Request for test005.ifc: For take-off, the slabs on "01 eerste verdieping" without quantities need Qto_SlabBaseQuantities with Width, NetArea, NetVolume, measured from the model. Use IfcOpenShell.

First a look at what the model holds.

```python
import ifcopenshell
import ifcopenshell.util.element
import ifcopenshell.util.unit

model = ifcopenshell.open("test005.ifc")
print(model.schema)
for unit_type in ("LENGTHUNIT", "AREAUNIT", "VOLUMEUNIT"):
    print(unit_type, ifcopenshell.util.unit.calculate_unit_scale(model, unit_type))
storey = next(s for s in model.by_type("IfcBuildingStorey") if s.Name == "01 eerste verdieping")
slabs = [e for e in ifcopenshell.util.element.get_decomposition(storey) if e.is_a("IfcSlab")]
for e in sorted(slabs, key=lambda e: e.id()):
    print(e.id(), e.is_a(), e.Name, list(ifcopenshell.util.element.get_psets(e, qtos_only=True)), sep=" | ")
```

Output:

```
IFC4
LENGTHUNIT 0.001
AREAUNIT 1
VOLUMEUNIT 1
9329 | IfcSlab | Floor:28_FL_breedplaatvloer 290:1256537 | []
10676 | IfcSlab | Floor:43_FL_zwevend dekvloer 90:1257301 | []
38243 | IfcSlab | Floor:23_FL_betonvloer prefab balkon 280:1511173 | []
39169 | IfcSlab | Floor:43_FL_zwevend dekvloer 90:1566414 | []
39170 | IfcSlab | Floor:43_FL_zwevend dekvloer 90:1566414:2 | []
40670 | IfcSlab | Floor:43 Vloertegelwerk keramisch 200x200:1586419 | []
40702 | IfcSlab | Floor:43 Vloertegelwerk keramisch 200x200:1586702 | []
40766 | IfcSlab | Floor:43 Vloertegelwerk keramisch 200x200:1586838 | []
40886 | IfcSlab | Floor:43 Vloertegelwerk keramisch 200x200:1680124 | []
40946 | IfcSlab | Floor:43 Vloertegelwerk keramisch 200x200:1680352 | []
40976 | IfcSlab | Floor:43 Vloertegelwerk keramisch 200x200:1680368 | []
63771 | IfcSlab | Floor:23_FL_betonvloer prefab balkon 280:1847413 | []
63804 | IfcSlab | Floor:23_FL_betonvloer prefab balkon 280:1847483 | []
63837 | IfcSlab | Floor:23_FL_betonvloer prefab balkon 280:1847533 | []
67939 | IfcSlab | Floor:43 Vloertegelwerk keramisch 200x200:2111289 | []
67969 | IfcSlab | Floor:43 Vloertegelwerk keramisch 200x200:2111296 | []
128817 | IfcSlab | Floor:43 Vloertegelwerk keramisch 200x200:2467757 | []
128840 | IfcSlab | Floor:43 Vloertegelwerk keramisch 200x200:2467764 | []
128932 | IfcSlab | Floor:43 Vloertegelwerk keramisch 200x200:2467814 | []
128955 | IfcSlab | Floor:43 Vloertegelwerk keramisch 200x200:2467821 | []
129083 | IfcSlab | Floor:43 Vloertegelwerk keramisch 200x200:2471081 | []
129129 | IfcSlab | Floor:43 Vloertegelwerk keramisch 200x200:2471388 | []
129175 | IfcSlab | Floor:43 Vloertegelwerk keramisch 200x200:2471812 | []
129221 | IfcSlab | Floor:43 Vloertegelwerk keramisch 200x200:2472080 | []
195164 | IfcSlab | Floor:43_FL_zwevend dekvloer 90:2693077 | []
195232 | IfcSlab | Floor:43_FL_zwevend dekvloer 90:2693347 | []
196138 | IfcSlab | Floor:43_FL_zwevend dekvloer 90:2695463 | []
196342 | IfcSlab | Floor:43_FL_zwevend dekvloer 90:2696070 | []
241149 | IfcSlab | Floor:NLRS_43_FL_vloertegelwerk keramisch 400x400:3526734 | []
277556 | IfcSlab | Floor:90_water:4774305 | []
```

```python
import ifcopenshell
import ifcopenshell.api.pset
import ifcopenshell.geom
import ifcopenshell.util.element
import ifcopenshell.util.shape
import ifcopenshell.util.unit

model = ifcopenshell.open("test005.ifc")
unit_scale = ifcopenshell.util.unit.calculate_unit_scale(model)
area_scale = ifcopenshell.util.unit.calculate_unit_scale(model, "AREAUNIT")
volume_scale = ifcopenshell.util.unit.calculate_unit_scale(model, "VOLUMEUNIT")
settings = ifcopenshell.geom.settings()

storey = next(s for s in model.by_type("IfcBuildingStorey") if s.Name == "01 eerste verdieping")
slabs = [e for e in ifcopenshell.util.element.get_decomposition(storey) if e.is_a("IfcSlab")]

for e in sorted(slabs, key=lambda e: e.id()):
    if ifcopenshell.util.element.get_psets(e, qtos_only=True, should_inherit=False):
        continue
    # Geometry comes back in metres, in the element's own axes.
    shape = ifcopenshell.geom.create_shape(settings, e)
    values = {
        "Width": ifcopenshell.util.shape.get_z(shape.geometry) / unit_scale,
        "NetArea": ifcopenshell.util.shape.get_footprint_area(shape.geometry) / area_scale,
        "NetVolume": ifcopenshell.util.shape.get_volume(shape.geometry) / volume_scale,
    }
    qto = ifcopenshell.api.pset.add_qto(model, product=e, name="Qto_SlabBaseQuantities")
    ifcopenshell.api.pset.edit_qto(model, qto=qto, properties=values)
    print(e.id(), {k: round(v, 3) for k, v in values.items()})

model.write("test005_updated.ifc")
```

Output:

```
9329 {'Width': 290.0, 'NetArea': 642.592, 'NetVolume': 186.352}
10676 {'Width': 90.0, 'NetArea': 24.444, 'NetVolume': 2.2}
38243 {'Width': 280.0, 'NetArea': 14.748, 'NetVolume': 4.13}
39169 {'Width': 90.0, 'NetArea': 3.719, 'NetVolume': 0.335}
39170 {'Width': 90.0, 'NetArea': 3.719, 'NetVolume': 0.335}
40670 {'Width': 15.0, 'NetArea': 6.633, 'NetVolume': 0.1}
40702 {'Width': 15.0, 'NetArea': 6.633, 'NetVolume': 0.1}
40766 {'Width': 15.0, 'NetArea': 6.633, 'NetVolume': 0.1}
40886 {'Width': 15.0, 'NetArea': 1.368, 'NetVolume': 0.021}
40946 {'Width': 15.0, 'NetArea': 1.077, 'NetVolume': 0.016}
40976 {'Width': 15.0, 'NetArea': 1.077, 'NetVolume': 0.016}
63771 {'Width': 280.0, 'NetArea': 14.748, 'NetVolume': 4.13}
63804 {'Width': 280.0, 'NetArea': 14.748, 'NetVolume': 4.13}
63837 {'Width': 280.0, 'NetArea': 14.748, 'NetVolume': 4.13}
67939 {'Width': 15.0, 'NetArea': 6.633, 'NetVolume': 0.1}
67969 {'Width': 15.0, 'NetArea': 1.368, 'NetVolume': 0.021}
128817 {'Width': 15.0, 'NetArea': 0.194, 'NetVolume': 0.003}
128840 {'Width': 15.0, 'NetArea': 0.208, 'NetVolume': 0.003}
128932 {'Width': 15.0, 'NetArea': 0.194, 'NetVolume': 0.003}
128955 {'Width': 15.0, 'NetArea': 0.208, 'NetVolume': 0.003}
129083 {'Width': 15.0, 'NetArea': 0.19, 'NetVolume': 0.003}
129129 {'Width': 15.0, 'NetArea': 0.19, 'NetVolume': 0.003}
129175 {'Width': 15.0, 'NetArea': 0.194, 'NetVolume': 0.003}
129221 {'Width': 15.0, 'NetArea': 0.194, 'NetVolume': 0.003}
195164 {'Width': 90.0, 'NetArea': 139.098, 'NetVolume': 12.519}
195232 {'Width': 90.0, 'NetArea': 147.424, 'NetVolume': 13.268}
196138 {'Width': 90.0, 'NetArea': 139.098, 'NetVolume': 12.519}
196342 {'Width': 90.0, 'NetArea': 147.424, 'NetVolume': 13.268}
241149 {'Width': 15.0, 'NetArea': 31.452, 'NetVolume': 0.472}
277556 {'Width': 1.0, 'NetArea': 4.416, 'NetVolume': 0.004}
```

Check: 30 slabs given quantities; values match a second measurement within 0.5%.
